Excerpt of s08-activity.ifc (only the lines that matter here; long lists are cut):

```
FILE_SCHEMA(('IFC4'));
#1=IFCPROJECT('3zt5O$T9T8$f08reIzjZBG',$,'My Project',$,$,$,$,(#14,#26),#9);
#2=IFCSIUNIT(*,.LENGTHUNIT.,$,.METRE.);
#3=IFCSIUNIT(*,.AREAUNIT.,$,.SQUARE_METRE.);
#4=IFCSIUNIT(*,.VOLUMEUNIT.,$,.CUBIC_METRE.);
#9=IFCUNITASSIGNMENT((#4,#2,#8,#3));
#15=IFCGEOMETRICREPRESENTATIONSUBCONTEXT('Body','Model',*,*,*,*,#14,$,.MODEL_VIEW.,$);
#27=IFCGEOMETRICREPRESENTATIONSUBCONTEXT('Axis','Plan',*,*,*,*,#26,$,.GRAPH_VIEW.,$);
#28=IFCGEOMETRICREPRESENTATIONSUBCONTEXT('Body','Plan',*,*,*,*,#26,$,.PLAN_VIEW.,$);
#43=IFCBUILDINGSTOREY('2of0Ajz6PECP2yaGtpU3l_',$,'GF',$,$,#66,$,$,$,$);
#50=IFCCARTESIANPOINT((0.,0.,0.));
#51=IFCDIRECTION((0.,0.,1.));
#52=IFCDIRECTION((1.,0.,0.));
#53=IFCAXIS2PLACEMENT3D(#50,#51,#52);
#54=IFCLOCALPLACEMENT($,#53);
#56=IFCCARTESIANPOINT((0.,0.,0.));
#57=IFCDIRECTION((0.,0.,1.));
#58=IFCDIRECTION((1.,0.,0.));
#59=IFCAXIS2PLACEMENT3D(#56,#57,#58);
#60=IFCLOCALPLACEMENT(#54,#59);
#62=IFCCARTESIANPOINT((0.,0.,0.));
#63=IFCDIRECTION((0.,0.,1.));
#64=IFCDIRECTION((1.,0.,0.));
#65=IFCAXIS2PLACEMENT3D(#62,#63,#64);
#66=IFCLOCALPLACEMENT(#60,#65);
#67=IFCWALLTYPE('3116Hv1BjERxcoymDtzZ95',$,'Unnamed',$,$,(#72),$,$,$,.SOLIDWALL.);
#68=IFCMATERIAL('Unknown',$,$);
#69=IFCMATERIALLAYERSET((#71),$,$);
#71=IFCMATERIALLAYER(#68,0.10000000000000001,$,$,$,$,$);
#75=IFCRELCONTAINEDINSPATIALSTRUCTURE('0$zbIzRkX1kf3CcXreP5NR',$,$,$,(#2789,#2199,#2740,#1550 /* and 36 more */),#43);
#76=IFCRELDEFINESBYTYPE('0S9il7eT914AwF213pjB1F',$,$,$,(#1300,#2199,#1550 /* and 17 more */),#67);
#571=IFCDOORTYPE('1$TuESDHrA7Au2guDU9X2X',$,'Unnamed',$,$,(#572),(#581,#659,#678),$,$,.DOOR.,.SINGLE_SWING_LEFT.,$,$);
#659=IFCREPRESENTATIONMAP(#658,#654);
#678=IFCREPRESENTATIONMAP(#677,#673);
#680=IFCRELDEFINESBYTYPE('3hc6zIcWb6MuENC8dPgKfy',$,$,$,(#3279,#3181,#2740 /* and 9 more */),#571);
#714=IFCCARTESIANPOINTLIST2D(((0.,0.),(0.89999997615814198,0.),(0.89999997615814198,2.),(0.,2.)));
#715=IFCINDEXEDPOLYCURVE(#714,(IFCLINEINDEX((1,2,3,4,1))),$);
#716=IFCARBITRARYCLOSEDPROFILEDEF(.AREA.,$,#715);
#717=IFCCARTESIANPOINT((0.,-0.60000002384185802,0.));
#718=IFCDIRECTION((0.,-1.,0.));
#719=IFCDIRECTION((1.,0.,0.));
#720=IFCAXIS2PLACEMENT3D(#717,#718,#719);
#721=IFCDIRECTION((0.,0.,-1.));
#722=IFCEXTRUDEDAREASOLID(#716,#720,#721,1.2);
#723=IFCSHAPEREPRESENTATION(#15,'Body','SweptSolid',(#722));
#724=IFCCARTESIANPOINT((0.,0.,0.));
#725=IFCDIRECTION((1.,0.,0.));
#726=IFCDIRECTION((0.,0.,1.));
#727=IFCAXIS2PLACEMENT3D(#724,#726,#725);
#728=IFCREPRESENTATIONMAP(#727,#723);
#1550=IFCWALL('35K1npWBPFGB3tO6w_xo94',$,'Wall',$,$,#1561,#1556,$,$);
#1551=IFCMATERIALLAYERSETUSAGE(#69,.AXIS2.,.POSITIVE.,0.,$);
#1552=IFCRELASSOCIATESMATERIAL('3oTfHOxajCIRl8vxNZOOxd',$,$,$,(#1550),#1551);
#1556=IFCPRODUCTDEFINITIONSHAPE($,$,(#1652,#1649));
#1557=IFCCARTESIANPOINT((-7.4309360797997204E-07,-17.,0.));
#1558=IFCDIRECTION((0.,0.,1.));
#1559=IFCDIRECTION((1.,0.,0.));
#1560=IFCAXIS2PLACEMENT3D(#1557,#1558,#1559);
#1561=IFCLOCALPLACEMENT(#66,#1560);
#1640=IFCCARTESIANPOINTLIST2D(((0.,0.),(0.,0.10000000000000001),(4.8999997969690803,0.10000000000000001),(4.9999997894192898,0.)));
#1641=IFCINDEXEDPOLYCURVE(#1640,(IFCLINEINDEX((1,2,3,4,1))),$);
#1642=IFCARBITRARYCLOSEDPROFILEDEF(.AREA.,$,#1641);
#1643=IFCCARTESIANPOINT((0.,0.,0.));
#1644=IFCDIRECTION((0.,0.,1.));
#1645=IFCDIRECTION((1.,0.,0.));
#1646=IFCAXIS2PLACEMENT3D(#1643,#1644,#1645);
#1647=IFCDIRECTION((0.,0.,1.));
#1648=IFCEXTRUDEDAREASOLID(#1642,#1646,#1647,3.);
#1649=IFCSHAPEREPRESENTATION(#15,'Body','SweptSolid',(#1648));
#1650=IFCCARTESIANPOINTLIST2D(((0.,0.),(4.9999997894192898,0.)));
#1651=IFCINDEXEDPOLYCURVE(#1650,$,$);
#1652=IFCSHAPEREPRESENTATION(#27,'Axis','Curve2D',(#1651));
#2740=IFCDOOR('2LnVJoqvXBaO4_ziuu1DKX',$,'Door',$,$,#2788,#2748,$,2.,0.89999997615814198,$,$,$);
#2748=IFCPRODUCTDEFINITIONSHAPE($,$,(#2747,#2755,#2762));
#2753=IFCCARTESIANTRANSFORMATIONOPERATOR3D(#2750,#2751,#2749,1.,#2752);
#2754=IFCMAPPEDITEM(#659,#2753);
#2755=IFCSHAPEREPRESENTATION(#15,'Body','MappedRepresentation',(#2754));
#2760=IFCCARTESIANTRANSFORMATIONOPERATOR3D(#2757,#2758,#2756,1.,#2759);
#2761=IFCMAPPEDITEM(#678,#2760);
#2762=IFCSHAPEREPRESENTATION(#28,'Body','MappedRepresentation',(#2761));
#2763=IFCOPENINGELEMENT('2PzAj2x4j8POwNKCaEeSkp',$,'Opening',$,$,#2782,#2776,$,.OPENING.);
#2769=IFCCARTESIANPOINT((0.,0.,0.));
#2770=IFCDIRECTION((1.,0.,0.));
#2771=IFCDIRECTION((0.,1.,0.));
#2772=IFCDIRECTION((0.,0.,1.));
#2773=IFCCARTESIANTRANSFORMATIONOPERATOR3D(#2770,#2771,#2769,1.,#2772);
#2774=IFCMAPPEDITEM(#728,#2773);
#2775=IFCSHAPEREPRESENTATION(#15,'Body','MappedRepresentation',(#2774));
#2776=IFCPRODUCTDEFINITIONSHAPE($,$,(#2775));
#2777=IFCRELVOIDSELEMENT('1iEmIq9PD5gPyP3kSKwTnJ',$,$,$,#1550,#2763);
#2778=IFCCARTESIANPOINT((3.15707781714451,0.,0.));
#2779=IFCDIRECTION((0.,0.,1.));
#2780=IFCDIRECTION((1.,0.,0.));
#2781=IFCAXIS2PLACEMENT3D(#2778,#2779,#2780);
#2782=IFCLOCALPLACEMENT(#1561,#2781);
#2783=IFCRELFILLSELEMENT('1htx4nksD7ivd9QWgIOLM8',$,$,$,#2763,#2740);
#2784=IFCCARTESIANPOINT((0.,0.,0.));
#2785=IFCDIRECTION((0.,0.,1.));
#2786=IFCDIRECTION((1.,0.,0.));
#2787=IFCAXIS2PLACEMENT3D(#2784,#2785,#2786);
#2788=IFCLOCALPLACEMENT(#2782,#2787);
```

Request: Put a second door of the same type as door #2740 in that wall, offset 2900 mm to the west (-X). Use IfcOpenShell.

```python
import ifcopenshell
import ifcopenshell.api.feature
import ifcopenshell.api.geometry
import ifcopenshell.api.root
import ifcopenshell.geom
import ifcopenshell.util.element
import ifcopenshell.util.placement
import ifcopenshell.util.shape

model = ifcopenshell.open("s08-activity.ifc")
settings = ifcopenshell.geom.settings()


def volume(element):
    """Net volume in cubic metres, openings subtracted."""
    shape = ifcopenshell.geom.create_shape(settings, element)
    return ifcopenshell.util.shape.get_volume(shape.geometry)


door = model.by_id(2740)
opening = door.FillsVoids[0].RelatingOpeningElement
wall = opening.VoidsElements[0].RelatingBuildingElement
before = volume(wall)
shift = ifcopenshell.util.placement.get_local_placement(wall.ObjectPlacement)[:3, 0] * -2.9

# copy_class copies the void relationship, type, container and properties, but no geometry.
new_opening = ifcopenshell.api.root.copy_class(model, product=opening)
new_opening.Representation = ifcopenshell.util.element.copy_deep(
    model, opening.Representation, exclude=["IfcGeometricRepresentationContext", "IfcRepresentationMap"]
)
new_door = ifcopenshell.api.root.copy_class(model, product=door)
new_door.Representation = ifcopenshell.util.element.copy_deep(
    model, door.Representation, exclude=["IfcGeometricRepresentationContext", "IfcRepresentationMap"]
)
ifcopenshell.api.feature.add_filling(model, opening=new_opening, element=new_door)

for old, new in ((opening, new_opening), (door, new_door)):
    matrix = ifcopenshell.util.placement.get_local_placement(old.ObjectPlacement)
    matrix[:3, 3] += shift
    ifcopenshell.api.geometry.edit_object_placement(model, product=new, matrix=matrix, is_si=False)

after = volume(wall)

print(f"wall volume {before:.3f} -> {after:.3f} m3")

model.write("s08-activity-out.ifc")
```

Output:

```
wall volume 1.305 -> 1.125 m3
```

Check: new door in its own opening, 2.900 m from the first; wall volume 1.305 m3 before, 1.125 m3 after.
